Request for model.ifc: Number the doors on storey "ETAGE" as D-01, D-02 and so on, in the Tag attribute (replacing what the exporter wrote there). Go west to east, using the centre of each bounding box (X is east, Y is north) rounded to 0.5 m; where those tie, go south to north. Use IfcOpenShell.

First a look at what the model holds.

```python
import ifcopenshell
import ifcopenshell.util.element
import ifcopenshell.util.placement

model = ifcopenshell.open("model.ifc")
print(model.schema)
storey = next(s for s in model.by_type("IfcBuildingStorey") if s.Name == "ETAGE")
doors = [e for e in ifcopenshell.util.element.get_decomposition(storey) if e.is_a("IfcDoor")]
for e in sorted(doors, key=lambda e: e.id()):
    origin = ifcopenshell.util.placement.get_local_placement(e.ObjectPlacement)[:3, 3]
    print(e.id(), e.Tag, e.Name, origin.round(2) + 0.0, sep=" | ")
```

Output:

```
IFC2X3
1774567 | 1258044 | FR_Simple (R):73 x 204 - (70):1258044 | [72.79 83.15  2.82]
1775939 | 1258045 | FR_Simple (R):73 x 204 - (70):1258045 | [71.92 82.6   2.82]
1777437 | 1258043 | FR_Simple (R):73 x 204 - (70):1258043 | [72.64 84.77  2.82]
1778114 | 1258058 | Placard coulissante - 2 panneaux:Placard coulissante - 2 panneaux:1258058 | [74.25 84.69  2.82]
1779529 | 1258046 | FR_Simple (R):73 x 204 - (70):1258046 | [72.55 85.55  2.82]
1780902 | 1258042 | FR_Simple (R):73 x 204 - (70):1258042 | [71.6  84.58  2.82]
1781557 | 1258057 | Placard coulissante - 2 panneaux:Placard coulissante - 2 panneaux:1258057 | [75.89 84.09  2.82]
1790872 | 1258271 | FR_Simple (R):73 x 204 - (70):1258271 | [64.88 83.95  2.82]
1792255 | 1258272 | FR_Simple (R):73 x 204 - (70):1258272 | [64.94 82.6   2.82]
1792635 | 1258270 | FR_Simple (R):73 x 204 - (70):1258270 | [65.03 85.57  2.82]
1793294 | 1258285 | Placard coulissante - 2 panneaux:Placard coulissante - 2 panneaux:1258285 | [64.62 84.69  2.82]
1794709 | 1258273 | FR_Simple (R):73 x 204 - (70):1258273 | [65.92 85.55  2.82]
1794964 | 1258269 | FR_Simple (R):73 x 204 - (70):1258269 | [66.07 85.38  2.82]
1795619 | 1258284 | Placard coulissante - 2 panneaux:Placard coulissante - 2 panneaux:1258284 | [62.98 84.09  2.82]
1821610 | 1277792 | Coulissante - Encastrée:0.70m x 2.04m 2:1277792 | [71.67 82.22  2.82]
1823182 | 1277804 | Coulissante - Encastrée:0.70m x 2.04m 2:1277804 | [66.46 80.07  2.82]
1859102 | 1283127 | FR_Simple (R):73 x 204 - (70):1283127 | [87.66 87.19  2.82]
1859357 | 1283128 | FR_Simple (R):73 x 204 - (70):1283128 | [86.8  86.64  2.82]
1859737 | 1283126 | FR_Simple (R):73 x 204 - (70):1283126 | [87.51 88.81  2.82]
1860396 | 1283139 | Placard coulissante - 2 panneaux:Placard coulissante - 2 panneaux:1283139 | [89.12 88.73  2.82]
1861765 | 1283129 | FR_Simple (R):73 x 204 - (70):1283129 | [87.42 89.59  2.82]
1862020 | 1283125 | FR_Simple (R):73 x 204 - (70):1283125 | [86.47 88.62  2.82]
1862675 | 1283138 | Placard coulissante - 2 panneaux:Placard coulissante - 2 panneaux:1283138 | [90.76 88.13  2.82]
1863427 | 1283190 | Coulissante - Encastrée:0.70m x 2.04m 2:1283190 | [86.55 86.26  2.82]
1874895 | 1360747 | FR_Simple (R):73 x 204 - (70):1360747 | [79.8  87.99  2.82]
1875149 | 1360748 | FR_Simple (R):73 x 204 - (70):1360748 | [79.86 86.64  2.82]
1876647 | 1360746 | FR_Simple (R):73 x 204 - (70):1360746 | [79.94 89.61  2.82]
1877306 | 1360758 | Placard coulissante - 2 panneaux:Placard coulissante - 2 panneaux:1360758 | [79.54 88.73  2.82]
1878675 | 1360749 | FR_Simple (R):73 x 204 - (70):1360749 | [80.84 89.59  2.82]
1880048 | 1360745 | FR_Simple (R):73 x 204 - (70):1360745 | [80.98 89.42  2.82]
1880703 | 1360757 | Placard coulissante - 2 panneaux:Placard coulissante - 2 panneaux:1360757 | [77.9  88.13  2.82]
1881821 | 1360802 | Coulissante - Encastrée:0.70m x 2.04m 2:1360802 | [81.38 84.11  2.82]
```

```python
import ifcopenshell
import ifcopenshell.geom
import ifcopenshell.util.element
import ifcopenshell.util.shape

model = ifcopenshell.open("model.ifc")
settings = ifcopenshell.geom.settings()
settings.set("use-world-coords", True)


def centre(element):
    shape = ifcopenshell.geom.create_shape(settings, element)
    return ifcopenshell.util.shape.get_bbox_centroid(shape.geometry)


storey = next(s for s in model.by_type("IfcBuildingStorey") if s.Name == "ETAGE")
doors = [e for e in ifcopenshell.util.element.get_decomposition(storey) if e.is_a("IfcDoor")]

# Insertion points can sit at a corner or the storey origin, so sort by the geometry (in metres).
centres = {e: centre(e) for e in doors}
doors.sort(key=lambda e: (round(centres[e][0] / 0.5), centres[e][1]))

for i, e in enumerate(doors, start=1):
    number = f"D-{i:02d}"
    e.Tag = number
    print(e.id(), number)

model.write("model_edited.ifc")
```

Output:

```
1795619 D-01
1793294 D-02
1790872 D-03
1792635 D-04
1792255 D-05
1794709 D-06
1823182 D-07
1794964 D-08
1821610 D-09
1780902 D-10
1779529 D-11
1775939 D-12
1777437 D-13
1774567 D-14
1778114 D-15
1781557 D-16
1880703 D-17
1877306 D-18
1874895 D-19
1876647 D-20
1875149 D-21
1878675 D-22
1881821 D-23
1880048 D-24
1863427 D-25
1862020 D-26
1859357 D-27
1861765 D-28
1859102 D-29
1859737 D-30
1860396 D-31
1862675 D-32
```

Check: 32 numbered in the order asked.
